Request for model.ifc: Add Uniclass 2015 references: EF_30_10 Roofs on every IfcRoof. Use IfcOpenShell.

First a look at what the model holds.

```python
import ifcopenshell

model = ifcopenshell.open("model.ifc")
print(model.schema)
print("classifications:", [c.Name for c in model.by_type("IfcClassification")])
for ifc_class in ("IfcDoor", "IfcRoof", "IfcStair", "IfcWall", "IfcWindow"):
    print(ifc_class, len(model.by_type(ifc_class)))
```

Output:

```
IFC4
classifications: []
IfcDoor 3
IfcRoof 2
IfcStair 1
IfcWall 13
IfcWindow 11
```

```python
import ifcopenshell
import ifcopenshell.api.classification

model = ifcopenshell.open("model.ifc")

system = ifcopenshell.api.classification.add_classification(model, classification="Uniclass 2015")

codes = {
    "IfcRoof": ("EF_30_10", "Roofs"),
}
for ifc_class, (code, name) in codes.items():
    products = model.by_type(ifc_class)
    ifcopenshell.api.classification.add_reference(
        model, products=products, classification=system, identification=code, name=name
    )
    print(code, len(products))

model.write("model_rev.ifc")
```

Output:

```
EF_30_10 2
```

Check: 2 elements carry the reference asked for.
